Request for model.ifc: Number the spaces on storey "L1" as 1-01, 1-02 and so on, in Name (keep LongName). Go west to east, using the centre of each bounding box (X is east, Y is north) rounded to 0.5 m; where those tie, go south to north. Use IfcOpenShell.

First a look at what the model holds.

```python
import ifcopenshell
import ifcopenshell.util.element
import ifcopenshell.util.placement

model = ifcopenshell.open("model.ifc")
print(model.schema)
storey = next(s for s in model.by_type("IfcBuildingStorey") if s.Name == "L1")
spaces = [e for e in ifcopenshell.util.element.get_decomposition(storey) if e.is_a("IfcSpace")]
for e in sorted(spaces, key=lambda e: e.id()):
    origin = ifcopenshell.util.placement.get_local_placement(e.ObjectPlacement)[:3, 3]
    print(e.id(), e.Name, e.LongName, origin.round(2) + 0.0, sep=" | ")
```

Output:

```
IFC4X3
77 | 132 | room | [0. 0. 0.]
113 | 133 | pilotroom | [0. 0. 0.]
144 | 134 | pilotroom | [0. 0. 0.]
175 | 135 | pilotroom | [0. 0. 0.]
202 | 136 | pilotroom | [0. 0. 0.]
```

```python
import ifcopenshell
import ifcopenshell.geom
import ifcopenshell.util.element
import ifcopenshell.util.shape

model = ifcopenshell.open("model.ifc")
settings = ifcopenshell.geom.settings()
settings.set("use-world-coords", True)


def centre(element):
    shape = ifcopenshell.geom.create_shape(settings, element)
    return ifcopenshell.util.shape.get_bbox_centroid(shape.geometry)


storey = next(s for s in model.by_type("IfcBuildingStorey") if s.Name == "L1")
spaces = [e for e in ifcopenshell.util.element.get_decomposition(storey) if e.is_a("IfcSpace")]

# Insertion points can sit at a corner or the storey origin, so sort by the geometry (in metres).
centres = {e: centre(e) for e in spaces}
spaces.sort(key=lambda e: (round(centres[e][0] / 0.5), centres[e][1]))

for i, e in enumerate(spaces, start=1):
    number = f"1-{i:02d}"
    e.Name = number
    print(e.id(), number)

model.write("model-out.ifc")
```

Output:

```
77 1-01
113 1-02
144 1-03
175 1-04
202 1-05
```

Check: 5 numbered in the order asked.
